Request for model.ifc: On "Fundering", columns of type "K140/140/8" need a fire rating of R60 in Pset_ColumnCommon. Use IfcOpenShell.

First a look at what the model holds.

```python
import ifcopenshell
import ifcopenshell.util.element

model = ifcopenshell.open("model.ifc")
print(model.schema)
storey = next(s for s in model.by_type("IfcBuildingStorey") if s.Name == "Fundering")
columns = [e for e in ifcopenshell.util.element.get_decomposition(storey) if e.is_a("IfcColumn")]
seen = {}
for e in columns:
    element_type = ifcopenshell.util.element.get_type(e)
    key = (element_type.Name if element_type != e and element_type else None, ifcopenshell.util.element.get_pset(e, "Pset_ColumnCommon", "FireRating"))
    seen[key] = seen.get(key, 0) + 1
for (name, value), count in sorted(seen.items(), key=str):
    print(count, "x", name, "|", value)
```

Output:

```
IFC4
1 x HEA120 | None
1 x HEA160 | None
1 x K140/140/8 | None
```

```python
import ifcopenshell
import ifcopenshell.api.pset
import ifcopenshell.util.element

model = ifcopenshell.open("model.ifc")

storey = next(s for s in model.by_type("IfcBuildingStorey") if s.Name == "Fundering")
columns = [e for e in ifcopenshell.util.element.get_decomposition(storey) if e.is_a("IfcColumn")]

count = 0
for e in columns:
    element_type = ifcopenshell.util.element.get_type(e)
    if element_type in (None, e) or element_type.Name != "K140/140/8":
        continue
    # add_pset returns the element's existing set when there is one.
    pset = ifcopenshell.api.pset.add_pset(model, product=e, name="Pset_ColumnCommon")
    ifcopenshell.api.pset.edit_pset(model, pset=pset, properties={"FireRating": "R60"})
    count += 1

print(count, "columns updated")

model.write("model_updated.ifc")
```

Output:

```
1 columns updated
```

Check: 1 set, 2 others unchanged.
